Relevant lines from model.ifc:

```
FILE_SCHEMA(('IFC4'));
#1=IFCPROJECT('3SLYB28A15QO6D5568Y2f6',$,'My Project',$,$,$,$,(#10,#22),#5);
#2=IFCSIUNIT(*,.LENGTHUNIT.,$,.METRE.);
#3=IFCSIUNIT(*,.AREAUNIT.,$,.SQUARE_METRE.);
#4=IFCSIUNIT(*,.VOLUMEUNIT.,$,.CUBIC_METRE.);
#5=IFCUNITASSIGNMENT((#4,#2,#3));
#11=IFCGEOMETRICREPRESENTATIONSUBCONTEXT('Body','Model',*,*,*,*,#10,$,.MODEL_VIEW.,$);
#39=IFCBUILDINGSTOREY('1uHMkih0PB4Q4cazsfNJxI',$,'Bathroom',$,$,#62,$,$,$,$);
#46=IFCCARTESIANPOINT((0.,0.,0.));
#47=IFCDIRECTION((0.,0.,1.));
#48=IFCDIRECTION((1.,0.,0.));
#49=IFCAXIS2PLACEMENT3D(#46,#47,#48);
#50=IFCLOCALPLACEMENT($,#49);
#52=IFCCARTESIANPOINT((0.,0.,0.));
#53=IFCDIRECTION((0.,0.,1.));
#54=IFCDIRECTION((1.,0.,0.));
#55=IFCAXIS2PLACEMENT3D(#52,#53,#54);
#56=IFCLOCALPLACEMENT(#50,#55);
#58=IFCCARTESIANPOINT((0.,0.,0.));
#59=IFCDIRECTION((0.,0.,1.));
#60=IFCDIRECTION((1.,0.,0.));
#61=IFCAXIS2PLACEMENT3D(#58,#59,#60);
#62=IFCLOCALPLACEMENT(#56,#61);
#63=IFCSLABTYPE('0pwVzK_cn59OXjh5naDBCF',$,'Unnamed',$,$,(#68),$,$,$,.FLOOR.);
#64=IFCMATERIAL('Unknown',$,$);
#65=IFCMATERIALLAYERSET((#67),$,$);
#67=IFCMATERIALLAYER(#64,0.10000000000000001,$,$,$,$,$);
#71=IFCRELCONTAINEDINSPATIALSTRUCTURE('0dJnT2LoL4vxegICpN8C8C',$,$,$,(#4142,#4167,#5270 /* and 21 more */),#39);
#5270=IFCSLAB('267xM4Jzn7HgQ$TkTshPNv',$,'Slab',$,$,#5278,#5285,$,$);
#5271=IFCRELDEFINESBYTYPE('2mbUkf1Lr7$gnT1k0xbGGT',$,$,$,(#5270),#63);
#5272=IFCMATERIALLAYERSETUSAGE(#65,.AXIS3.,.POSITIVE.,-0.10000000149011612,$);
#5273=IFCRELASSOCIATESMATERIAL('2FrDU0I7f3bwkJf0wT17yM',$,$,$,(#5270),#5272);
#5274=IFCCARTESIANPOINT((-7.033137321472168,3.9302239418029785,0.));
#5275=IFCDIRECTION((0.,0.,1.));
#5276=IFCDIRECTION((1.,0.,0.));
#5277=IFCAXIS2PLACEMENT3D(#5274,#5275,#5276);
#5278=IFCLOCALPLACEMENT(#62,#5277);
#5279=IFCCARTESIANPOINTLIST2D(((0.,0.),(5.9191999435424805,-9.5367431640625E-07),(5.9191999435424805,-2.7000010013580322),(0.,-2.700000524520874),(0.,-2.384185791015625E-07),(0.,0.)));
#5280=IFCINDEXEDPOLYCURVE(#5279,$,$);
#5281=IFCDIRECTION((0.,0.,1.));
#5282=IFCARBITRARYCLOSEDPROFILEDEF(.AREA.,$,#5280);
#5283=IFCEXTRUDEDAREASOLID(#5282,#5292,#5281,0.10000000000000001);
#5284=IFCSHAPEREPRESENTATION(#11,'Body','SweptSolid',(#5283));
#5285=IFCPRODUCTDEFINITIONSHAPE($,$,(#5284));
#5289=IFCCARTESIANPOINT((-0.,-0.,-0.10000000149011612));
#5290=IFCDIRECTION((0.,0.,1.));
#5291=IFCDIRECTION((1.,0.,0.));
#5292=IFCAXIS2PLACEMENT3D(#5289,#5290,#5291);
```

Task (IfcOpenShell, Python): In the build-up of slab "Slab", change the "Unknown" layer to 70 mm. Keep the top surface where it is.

```python
import ifcopenshell
import ifcopenshell.util.element
import ifcopenshell.util.representation

model = ifcopenshell.open("model.ifc")

layer_set = model.by_id(65)
layer = next(l for l in layer_set.MaterialLayers if l.Material and l.Material.Name == "Unknown")
change = 0.07 - layer.LayerThickness
layer.LayerThickness += change

# Geometry does not follow the layer set by itself.
slabs = [e for e in ifcopenshell.util.element.get_elements_by_material(model, layer_set) if e.is_a("IfcSlab")]
for slab in sorted(slabs, key=lambda e: e.id()):
    body = ifcopenshell.util.representation.get_representation(slab, "Model", "Body")
    solid = body.Items[0]
    old_depth = solid.Depth
    solid.Depth += change
    # Extruded upwards: lower the start of the extrusion so the top stays.
    x, y, z = solid.Position.Location.Coordinates
    solid.Position.Location = model.createIfcCartesianPoint((x, y, z - change))
    print(slab.id(), f"{old_depth:g} -> {solid.Depth:g}")

# The layers are counted up from the underside, which has moved.
for usage in {ifcopenshell.util.element.get_material(slab) for slab in slabs}:
    usage.OffsetFromReferenceLine -= change

model.write("model_rev.ifc")
```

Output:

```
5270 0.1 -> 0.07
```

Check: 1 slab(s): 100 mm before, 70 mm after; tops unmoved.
